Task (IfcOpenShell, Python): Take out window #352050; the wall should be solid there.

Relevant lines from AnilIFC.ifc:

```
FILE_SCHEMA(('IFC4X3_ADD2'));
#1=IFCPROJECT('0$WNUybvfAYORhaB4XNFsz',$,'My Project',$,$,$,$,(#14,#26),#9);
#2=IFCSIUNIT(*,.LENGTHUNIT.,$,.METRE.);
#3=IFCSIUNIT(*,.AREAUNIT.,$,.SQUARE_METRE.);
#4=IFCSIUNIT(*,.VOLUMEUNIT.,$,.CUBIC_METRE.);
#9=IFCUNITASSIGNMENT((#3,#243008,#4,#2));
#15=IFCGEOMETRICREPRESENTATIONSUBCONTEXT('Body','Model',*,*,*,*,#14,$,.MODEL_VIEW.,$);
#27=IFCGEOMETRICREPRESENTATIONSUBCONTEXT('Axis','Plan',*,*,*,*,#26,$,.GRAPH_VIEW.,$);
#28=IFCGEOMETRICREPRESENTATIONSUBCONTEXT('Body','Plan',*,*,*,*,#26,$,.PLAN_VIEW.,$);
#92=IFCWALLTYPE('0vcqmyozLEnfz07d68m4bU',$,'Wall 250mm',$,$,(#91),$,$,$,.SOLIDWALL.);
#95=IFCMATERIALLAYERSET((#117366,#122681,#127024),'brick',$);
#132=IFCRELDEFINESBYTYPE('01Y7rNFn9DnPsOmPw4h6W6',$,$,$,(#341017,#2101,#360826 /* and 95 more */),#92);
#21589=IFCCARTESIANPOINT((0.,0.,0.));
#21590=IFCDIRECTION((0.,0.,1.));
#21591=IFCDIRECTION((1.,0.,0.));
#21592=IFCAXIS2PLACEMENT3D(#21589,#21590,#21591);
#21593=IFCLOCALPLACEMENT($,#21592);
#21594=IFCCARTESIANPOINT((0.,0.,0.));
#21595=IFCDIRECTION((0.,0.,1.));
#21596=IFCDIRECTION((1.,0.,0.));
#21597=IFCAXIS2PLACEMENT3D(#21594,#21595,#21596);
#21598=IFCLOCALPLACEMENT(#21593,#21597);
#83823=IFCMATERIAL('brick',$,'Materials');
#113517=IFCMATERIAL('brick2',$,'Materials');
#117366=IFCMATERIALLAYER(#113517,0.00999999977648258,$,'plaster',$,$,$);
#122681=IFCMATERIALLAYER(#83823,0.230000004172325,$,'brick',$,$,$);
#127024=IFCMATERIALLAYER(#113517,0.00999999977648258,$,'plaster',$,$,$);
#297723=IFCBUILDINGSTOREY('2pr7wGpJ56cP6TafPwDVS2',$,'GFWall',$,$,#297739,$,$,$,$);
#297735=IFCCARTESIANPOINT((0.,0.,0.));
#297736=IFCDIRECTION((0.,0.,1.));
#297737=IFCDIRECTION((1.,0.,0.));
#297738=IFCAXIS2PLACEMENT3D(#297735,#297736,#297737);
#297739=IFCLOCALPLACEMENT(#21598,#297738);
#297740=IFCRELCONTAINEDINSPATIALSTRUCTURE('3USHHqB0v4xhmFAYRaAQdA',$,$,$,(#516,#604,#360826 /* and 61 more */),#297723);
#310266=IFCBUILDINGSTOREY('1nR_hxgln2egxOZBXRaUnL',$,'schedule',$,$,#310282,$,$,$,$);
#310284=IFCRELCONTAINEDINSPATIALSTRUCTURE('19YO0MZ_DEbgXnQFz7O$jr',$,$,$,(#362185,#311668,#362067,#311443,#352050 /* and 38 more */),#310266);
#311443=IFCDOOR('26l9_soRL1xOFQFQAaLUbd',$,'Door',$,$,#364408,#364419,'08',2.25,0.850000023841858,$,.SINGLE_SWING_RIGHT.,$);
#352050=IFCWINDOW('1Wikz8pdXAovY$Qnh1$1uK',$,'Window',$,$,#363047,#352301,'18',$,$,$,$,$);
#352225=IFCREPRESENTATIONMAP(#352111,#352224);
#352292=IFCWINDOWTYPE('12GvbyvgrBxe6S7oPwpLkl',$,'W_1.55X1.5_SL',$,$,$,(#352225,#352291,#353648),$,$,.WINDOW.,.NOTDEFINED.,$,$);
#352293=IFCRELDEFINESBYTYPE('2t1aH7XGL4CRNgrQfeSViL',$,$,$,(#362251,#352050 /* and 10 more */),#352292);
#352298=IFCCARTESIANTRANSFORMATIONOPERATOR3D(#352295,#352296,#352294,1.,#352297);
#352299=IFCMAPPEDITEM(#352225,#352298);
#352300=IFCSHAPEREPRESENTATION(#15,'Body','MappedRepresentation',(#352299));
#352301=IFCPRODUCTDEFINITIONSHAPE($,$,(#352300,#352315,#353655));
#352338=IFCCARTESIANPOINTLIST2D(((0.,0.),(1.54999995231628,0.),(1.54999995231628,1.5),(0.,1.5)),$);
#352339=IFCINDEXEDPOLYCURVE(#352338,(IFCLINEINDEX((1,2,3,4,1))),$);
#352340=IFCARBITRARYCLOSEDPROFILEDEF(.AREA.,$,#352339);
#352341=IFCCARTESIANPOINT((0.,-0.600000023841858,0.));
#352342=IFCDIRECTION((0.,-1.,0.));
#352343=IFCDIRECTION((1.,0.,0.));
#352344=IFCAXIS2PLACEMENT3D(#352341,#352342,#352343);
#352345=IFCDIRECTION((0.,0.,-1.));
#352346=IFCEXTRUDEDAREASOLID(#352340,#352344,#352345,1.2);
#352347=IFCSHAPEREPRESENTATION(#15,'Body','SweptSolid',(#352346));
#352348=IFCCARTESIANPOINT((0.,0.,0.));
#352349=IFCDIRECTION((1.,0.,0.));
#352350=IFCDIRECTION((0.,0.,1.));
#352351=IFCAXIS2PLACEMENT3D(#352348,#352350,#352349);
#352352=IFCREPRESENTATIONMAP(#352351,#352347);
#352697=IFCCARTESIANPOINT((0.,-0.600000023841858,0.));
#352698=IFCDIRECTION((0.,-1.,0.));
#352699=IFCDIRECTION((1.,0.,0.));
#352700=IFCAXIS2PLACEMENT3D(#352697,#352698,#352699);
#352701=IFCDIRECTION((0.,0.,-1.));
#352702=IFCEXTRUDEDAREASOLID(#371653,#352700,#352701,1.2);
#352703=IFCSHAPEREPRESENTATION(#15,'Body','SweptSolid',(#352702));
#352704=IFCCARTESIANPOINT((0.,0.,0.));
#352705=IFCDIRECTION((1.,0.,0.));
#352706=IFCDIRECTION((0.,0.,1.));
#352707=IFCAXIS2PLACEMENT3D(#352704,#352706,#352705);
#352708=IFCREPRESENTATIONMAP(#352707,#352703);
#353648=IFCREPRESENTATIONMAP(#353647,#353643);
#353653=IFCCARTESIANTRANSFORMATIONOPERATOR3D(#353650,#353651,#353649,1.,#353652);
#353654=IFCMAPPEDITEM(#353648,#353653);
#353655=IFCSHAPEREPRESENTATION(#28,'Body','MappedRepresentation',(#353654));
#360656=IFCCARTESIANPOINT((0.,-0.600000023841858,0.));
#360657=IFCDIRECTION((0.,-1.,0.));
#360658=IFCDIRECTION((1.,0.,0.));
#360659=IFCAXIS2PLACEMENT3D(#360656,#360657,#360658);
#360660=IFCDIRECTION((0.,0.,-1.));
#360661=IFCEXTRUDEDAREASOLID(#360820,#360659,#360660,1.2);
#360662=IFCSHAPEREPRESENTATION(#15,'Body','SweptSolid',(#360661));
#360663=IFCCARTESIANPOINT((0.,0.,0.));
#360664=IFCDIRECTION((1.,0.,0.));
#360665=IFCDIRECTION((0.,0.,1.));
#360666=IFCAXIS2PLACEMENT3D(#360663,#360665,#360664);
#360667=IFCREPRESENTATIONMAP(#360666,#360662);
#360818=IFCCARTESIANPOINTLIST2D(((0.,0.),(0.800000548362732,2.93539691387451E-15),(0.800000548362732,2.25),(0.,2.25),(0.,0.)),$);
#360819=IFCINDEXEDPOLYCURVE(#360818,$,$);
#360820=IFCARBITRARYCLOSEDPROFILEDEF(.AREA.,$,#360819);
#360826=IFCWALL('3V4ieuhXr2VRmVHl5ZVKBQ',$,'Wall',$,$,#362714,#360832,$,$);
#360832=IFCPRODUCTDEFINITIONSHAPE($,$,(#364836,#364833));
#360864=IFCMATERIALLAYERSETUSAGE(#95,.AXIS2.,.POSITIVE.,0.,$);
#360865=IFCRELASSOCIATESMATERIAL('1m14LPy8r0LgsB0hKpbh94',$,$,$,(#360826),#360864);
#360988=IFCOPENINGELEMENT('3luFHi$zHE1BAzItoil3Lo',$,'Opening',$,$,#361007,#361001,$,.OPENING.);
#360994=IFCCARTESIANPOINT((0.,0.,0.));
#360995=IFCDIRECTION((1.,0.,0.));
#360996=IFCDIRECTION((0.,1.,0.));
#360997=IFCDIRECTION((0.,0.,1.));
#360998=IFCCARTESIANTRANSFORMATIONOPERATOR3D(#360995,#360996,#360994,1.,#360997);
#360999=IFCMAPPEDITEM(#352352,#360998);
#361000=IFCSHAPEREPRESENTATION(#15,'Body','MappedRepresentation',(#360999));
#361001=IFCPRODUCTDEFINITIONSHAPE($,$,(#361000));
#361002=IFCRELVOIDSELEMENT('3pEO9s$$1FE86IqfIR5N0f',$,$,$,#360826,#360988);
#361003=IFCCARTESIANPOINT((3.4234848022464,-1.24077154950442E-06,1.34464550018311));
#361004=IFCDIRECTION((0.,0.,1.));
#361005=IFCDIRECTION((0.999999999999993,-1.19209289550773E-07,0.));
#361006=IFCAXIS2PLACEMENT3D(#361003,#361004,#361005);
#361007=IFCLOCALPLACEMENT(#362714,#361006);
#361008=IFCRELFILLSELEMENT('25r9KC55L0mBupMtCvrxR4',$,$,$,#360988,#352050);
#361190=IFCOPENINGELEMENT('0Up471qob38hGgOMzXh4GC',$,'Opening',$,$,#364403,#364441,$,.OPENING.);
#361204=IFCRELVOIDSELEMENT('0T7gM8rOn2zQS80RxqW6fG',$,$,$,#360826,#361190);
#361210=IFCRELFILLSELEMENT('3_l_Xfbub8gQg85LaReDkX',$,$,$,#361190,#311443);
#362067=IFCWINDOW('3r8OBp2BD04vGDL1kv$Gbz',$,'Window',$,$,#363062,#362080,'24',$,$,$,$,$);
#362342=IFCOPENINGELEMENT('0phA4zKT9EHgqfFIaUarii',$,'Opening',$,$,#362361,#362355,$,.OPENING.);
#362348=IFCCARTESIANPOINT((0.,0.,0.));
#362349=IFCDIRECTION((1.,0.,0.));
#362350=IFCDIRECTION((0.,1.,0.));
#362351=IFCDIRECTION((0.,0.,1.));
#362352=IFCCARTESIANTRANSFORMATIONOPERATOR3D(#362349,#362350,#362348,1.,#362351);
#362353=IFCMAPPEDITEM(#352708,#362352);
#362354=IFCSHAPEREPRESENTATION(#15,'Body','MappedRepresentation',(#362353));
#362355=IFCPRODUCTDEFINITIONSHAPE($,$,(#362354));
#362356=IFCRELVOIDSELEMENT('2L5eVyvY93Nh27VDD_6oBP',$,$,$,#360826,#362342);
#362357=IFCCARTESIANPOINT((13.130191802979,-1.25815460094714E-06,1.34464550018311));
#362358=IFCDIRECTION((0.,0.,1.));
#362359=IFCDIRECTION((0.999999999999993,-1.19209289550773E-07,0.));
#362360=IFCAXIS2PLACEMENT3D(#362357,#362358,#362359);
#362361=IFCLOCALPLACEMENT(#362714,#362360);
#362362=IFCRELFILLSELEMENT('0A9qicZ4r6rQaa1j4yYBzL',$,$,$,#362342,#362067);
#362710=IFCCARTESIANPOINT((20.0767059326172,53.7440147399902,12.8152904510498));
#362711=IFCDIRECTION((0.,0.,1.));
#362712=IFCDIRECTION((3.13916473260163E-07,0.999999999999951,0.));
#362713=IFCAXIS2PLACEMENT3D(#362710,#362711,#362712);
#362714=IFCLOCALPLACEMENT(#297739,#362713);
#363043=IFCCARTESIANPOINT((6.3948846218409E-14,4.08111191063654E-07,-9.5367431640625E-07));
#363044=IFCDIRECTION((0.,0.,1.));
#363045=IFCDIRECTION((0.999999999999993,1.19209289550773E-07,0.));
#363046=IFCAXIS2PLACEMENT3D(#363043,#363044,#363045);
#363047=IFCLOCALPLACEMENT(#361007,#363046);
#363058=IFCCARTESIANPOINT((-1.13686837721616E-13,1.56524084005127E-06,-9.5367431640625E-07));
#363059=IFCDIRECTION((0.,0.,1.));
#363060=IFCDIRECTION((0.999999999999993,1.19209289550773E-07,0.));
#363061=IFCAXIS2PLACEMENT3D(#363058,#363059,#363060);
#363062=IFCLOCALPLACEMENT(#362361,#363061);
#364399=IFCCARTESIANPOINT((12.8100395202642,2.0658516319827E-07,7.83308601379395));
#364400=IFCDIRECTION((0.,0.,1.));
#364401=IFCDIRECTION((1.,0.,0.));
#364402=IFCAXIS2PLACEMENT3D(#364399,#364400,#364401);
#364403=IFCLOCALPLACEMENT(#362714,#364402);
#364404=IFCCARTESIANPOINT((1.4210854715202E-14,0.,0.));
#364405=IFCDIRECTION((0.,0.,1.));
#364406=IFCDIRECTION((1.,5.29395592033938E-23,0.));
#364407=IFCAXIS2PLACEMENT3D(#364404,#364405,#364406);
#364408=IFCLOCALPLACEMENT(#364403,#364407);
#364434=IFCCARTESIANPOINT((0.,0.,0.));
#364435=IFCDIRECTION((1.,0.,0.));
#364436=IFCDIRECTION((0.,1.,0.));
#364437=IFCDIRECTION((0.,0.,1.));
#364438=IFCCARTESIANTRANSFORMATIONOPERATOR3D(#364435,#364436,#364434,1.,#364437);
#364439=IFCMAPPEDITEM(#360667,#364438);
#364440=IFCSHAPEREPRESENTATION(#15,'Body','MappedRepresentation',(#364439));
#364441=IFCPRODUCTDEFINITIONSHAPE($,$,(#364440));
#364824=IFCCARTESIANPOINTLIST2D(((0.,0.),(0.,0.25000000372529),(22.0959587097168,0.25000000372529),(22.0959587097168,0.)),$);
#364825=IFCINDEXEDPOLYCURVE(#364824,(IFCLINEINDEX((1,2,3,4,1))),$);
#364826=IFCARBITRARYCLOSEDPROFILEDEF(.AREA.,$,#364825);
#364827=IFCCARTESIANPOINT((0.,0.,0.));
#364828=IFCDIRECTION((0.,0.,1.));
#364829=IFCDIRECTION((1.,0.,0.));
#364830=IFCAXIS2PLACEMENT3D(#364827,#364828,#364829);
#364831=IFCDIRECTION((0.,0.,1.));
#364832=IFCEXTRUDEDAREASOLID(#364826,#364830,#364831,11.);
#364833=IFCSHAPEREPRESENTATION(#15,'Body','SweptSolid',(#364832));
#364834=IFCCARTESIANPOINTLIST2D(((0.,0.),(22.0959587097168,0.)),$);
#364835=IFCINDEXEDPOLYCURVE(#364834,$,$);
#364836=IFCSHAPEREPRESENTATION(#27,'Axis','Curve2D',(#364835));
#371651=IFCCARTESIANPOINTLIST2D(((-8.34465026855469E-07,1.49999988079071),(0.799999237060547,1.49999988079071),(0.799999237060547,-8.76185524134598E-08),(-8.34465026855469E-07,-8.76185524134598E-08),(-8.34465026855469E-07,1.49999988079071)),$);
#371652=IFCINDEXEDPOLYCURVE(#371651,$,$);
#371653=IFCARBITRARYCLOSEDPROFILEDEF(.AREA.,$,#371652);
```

```python
import ifcopenshell
import ifcopenshell.api.feature
import ifcopenshell.api.root
import ifcopenshell.geom
import ifcopenshell.util.shape

model = ifcopenshell.open("AnilIFC.ifc")
settings = ifcopenshell.geom.settings()


def volume(element):
    """Net volume in cubic metres, openings subtracted."""
    shape = ifcopenshell.geom.create_shape(settings, element)
    return ifcopenshell.util.shape.get_volume(shape.geometry)


window = model.by_guid("1Wikz8pdXAovY$Qnh1$1uK")
opening = window.FillsVoids[0].RelatingOpeningElement
wall = opening.VoidsElements[0].RelatingBuildingElement
before = volume(wall)

ifcopenshell.api.root.remove_product(model, product=window)
ifcopenshell.api.feature.remove_feature(model, feature=opening)

after = volume(wall)

print(f"wall volume {before:.3f} -> {after:.3f} m3")

model.write("AnilIFC_edited.ifc")
```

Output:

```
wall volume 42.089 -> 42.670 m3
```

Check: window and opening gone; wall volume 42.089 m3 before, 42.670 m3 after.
